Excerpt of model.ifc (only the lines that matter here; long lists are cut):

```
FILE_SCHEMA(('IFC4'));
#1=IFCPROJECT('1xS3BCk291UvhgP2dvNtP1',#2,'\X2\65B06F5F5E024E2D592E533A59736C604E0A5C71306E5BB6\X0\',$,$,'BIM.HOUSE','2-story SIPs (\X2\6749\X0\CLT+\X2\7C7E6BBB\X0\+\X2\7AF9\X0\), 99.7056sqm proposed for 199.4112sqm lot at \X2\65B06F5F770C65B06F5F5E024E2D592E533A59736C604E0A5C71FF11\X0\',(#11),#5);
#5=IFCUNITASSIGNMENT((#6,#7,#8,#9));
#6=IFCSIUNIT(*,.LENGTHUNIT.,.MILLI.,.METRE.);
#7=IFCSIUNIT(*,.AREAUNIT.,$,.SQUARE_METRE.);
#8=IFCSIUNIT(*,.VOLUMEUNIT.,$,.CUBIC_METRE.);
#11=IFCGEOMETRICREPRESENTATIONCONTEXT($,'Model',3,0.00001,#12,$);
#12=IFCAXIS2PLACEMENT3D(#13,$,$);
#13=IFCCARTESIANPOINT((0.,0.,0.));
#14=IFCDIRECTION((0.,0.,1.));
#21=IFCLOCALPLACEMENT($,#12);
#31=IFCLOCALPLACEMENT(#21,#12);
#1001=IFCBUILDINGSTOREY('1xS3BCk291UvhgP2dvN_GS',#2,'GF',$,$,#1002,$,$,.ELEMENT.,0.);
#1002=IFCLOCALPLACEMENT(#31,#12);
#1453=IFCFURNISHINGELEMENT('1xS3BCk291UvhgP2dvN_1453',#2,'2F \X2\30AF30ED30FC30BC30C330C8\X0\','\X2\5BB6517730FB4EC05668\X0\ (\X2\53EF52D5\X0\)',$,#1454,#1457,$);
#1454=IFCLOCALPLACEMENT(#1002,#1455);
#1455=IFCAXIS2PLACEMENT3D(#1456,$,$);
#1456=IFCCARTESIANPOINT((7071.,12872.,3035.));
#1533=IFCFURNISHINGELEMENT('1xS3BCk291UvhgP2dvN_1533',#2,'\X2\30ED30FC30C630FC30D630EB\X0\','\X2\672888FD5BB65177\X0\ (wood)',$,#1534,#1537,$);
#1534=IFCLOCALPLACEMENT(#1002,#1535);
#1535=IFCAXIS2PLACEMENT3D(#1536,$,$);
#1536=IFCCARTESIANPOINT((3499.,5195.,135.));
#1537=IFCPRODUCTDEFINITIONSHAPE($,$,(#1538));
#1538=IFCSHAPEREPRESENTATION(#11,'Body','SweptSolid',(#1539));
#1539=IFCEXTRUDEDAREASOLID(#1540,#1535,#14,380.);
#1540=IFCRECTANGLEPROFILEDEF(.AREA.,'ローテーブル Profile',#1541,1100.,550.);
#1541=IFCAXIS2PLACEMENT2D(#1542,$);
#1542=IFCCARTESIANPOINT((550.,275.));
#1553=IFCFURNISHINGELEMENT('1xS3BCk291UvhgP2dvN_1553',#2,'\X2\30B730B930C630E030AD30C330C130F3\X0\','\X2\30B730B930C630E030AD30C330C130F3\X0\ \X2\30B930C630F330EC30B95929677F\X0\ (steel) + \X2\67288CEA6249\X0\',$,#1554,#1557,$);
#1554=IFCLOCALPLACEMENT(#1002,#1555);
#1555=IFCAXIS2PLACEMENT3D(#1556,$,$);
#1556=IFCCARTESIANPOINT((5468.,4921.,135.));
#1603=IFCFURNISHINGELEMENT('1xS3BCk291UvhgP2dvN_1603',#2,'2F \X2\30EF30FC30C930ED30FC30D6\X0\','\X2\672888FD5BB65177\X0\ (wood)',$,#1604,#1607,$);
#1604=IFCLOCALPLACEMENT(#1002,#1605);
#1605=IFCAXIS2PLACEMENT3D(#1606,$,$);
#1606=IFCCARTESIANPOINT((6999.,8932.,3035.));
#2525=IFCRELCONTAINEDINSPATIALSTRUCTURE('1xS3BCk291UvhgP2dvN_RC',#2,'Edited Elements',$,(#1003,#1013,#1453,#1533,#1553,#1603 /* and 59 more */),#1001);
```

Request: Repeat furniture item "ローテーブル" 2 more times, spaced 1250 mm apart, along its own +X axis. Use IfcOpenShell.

```python
import ifcopenshell
import ifcopenshell.api.geometry
import ifcopenshell.api.root
import ifcopenshell.util.element
import ifcopenshell.util.placement
import ifcopenshell.util.unit

model = ifcopenshell.open("model.ifc")
unit_scale = ifcopenshell.util.unit.calculate_unit_scale(model)


def reuse_history(source, copy):
    """copy_class also copies each property set's owner history, people and application; keep the originals."""
    for rel in copy.IsDefinedBy:
        if rel.is_a("IfcRelDefinesByProperties") and (history := rel.RelatingPropertyDefinition.OwnerHistory):
            rel.RelatingPropertyDefinition.OwnerHistory = source.OwnerHistory
            ifcopenshell.util.element.remove_deep2(model, history)


source = model.by_guid("1xS3BCk291UvhgP2dvN_1533")
base = ifcopenshell.util.placement.get_local_placement(source.ObjectPlacement)
step = base[:3, 0] * 1.25 / unit_scale

for i in range(1, 3):
    copy = ifcopenshell.api.root.copy_class(model, product=source)
    copy.Representation = ifcopenshell.util.element.copy_deep(
        model, source.Representation, exclude=["IfcGeometricRepresentationContext", "IfcRepresentationMap"]
    )
    reuse_history(source, copy)
    matrix = base.copy()
    matrix[:3, 3] += i * step
    print("added at", matrix[:3, 3].round(3) + 0.0)
    ifcopenshell.api.geometry.edit_object_placement(model, product=copy, matrix=matrix, is_si=False)

model.write("model_rev.ifc")
```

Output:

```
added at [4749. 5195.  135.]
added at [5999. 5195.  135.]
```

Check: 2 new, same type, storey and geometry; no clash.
